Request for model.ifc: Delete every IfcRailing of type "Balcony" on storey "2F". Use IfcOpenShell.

First a look at what the model holds.

```python
import ifcopenshell
import ifcopenshell.util.element

model = ifcopenshell.open("model.ifc")
print(model.schema)
storey = next(s for s in model.by_type("IfcBuildingStorey") if s.Name == "2F")
railings = [e for e in ifcopenshell.util.element.get_decomposition(storey) if e.is_a("IfcRailing")]
seen = {}
for e in railings:
    element_type = ifcopenshell.util.element.get_type(e)
    name = element_type.Name if element_type not in (None, e) else None
    seen[name] = seen.get(name, 0) + 1
for name, count in sorted(seen.items(), key=str):
    print(count, "x", name)
```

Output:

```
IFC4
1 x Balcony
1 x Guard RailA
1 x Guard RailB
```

```python
import ifcopenshell
import ifcopenshell.api.root
import ifcopenshell.util.element

model = ifcopenshell.open("model.ifc")

storey = next(s for s in model.by_type("IfcBuildingStorey") if s.Name == "2F")
railings = [e for e in ifcopenshell.util.element.get_decomposition(storey) if e.is_a("IfcRailing")]
targets = [e for e in railings if (t := ifcopenshell.util.element.get_type(e)) not in (None, e) and t.Name == "Balcony"]

for e in targets:
    ifcopenshell.api.root.remove_product(model, product=e)
print(len(targets), "removed")

model.write("model_v2.ifc")
```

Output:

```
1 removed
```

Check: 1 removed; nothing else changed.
